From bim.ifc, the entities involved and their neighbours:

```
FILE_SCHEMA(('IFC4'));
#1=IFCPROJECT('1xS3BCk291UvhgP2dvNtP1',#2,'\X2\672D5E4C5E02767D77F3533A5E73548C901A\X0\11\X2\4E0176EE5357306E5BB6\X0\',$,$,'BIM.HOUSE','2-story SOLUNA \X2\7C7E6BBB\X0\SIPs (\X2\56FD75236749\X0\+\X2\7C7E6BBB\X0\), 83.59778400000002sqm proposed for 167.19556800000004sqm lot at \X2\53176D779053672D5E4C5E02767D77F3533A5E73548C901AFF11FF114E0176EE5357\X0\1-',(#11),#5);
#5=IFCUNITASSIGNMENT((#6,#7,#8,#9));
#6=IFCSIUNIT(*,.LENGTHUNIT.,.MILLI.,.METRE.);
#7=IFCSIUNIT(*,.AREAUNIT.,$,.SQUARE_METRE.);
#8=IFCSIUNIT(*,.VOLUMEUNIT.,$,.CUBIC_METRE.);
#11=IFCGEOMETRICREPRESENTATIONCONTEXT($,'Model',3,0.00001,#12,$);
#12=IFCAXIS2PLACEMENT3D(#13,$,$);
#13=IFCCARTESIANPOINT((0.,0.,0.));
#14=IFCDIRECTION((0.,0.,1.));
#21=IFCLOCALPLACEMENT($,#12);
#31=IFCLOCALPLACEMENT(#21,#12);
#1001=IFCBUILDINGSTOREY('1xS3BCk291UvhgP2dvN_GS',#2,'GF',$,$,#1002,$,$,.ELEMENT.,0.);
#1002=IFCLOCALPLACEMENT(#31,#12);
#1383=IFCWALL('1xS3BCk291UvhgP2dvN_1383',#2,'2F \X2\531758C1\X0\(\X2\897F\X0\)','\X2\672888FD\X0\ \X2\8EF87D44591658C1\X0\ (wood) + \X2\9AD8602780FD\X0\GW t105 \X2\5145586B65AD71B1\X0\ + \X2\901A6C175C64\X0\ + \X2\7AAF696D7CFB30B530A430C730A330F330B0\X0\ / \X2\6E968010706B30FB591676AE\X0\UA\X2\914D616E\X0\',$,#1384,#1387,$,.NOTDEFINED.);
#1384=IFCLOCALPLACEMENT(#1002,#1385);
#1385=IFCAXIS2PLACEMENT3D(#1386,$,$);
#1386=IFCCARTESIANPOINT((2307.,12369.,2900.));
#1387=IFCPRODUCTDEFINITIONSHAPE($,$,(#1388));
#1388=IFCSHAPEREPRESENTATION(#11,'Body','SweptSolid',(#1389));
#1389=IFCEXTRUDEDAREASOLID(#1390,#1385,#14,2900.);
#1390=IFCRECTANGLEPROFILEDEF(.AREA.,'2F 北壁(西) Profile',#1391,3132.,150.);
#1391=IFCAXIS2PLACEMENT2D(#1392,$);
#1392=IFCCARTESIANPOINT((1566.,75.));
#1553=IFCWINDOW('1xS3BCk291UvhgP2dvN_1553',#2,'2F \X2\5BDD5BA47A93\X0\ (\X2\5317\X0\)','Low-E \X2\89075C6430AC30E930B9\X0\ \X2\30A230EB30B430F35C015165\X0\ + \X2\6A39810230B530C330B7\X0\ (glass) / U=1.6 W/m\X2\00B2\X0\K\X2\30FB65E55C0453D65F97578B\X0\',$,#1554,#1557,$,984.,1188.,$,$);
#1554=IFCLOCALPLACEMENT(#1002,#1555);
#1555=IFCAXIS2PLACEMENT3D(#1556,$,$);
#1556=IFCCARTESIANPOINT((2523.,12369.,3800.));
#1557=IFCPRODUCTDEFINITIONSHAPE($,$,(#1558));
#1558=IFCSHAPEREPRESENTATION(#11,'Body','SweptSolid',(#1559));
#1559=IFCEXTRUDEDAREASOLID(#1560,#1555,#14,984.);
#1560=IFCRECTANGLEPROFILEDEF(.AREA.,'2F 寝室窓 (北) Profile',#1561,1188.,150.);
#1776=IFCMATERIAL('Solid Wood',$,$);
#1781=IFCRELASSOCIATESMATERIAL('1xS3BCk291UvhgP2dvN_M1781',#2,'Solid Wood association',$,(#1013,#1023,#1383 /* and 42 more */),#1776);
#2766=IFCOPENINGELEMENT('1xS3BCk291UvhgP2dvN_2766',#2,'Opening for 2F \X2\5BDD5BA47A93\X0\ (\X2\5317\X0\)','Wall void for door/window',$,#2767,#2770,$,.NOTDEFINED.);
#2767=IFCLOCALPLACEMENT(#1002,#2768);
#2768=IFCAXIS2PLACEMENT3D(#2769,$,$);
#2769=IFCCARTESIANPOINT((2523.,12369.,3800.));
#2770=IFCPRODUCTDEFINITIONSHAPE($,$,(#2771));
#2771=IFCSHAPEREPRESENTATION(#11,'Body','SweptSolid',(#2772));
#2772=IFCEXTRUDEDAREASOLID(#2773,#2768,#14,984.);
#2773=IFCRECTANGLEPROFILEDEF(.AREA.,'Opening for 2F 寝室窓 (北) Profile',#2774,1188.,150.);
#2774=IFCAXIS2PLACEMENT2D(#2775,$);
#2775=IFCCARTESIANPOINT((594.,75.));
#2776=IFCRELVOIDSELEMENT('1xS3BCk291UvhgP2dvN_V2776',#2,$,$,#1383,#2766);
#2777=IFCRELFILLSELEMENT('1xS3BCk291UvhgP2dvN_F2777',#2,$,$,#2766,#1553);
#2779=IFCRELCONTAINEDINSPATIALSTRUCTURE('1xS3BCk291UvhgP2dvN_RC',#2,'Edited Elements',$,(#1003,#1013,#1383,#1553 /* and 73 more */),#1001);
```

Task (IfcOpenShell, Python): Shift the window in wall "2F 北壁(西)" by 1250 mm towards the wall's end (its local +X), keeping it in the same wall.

```python
import ifcopenshell
import ifcopenshell.api.geometry
import ifcopenshell.util.placement

model = ifcopenshell.open("bim.ifc")

window = model.by_guid("1xS3BCk291UvhgP2dvN_1553")
opening = window.FillsVoids[0].RelatingOpeningElement
wall = opening.VoidsElements[0].RelatingBuildingElement

wall_matrix = ifcopenshell.util.placement.get_local_placement(wall.ObjectPlacement)
shift = wall_matrix[:3, 0] * 1250.0
before = ifcopenshell.util.placement.get_local_placement(window.ObjectPlacement)[:3, 3].copy()

# The window is not placed relative to its opening, so move both.
for product in (opening, window):
    matrix = ifcopenshell.util.placement.get_local_placement(product.ObjectPlacement)
    matrix[:3, 3] += shift
    ifcopenshell.api.geometry.edit_object_placement(model, product=product, matrix=matrix, is_si=False)

after = ifcopenshell.util.placement.get_local_placement(window.ObjectPlacement)[:3, 3]
print("window moved by", (after - before).round(3) + 0.0)

model.write("bim_edited.ifc")
```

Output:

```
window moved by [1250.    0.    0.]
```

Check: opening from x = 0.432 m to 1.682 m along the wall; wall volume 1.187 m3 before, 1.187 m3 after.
